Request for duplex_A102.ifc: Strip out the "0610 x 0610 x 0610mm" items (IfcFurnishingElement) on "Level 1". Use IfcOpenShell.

First a look at what the model holds.

```python
import ifcopenshell
import ifcopenshell.util.element

model = ifcopenshell.open("duplex_A102.ifc")
print(model.schema)
storey = next(s for s in model.by_type("IfcBuildingStorey") if s.Name == "Level 1")
furniture = [e for e in ifcopenshell.util.element.get_decomposition(storey) if e.is_a("IfcFurnishingElement")]
seen = {}
for e in furniture:
    element_type = ifcopenshell.util.element.get_type(e)
    name = element_type.Name if element_type not in (None, e) else None
    seen[name] = seen.get(name, 0) + 1
for name, count in sorted(seen.items(), key=str):
    print(count, "x", name)
```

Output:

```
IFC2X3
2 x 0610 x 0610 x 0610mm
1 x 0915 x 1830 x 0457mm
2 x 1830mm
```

```python
import ifcopenshell
import ifcopenshell.api.root
import ifcopenshell.util.element

model = ifcopenshell.open("duplex_A102.ifc")

storey = next(s for s in model.by_type("IfcBuildingStorey") if s.Name == "Level 1")
furniture = [e for e in ifcopenshell.util.element.get_decomposition(storey) if e.is_a("IfcFurnishingElement")]
targets = [e for e in furniture if (t := ifcopenshell.util.element.get_type(e)) not in (None, e) and t.Name == "0610 x 0610 x 0610mm"]

for e in targets:
    ifcopenshell.api.root.remove_product(model, product=e)
print(len(targets), "removed")

model.write("duplex_A102-out.ifc")
```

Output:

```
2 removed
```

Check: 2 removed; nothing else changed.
